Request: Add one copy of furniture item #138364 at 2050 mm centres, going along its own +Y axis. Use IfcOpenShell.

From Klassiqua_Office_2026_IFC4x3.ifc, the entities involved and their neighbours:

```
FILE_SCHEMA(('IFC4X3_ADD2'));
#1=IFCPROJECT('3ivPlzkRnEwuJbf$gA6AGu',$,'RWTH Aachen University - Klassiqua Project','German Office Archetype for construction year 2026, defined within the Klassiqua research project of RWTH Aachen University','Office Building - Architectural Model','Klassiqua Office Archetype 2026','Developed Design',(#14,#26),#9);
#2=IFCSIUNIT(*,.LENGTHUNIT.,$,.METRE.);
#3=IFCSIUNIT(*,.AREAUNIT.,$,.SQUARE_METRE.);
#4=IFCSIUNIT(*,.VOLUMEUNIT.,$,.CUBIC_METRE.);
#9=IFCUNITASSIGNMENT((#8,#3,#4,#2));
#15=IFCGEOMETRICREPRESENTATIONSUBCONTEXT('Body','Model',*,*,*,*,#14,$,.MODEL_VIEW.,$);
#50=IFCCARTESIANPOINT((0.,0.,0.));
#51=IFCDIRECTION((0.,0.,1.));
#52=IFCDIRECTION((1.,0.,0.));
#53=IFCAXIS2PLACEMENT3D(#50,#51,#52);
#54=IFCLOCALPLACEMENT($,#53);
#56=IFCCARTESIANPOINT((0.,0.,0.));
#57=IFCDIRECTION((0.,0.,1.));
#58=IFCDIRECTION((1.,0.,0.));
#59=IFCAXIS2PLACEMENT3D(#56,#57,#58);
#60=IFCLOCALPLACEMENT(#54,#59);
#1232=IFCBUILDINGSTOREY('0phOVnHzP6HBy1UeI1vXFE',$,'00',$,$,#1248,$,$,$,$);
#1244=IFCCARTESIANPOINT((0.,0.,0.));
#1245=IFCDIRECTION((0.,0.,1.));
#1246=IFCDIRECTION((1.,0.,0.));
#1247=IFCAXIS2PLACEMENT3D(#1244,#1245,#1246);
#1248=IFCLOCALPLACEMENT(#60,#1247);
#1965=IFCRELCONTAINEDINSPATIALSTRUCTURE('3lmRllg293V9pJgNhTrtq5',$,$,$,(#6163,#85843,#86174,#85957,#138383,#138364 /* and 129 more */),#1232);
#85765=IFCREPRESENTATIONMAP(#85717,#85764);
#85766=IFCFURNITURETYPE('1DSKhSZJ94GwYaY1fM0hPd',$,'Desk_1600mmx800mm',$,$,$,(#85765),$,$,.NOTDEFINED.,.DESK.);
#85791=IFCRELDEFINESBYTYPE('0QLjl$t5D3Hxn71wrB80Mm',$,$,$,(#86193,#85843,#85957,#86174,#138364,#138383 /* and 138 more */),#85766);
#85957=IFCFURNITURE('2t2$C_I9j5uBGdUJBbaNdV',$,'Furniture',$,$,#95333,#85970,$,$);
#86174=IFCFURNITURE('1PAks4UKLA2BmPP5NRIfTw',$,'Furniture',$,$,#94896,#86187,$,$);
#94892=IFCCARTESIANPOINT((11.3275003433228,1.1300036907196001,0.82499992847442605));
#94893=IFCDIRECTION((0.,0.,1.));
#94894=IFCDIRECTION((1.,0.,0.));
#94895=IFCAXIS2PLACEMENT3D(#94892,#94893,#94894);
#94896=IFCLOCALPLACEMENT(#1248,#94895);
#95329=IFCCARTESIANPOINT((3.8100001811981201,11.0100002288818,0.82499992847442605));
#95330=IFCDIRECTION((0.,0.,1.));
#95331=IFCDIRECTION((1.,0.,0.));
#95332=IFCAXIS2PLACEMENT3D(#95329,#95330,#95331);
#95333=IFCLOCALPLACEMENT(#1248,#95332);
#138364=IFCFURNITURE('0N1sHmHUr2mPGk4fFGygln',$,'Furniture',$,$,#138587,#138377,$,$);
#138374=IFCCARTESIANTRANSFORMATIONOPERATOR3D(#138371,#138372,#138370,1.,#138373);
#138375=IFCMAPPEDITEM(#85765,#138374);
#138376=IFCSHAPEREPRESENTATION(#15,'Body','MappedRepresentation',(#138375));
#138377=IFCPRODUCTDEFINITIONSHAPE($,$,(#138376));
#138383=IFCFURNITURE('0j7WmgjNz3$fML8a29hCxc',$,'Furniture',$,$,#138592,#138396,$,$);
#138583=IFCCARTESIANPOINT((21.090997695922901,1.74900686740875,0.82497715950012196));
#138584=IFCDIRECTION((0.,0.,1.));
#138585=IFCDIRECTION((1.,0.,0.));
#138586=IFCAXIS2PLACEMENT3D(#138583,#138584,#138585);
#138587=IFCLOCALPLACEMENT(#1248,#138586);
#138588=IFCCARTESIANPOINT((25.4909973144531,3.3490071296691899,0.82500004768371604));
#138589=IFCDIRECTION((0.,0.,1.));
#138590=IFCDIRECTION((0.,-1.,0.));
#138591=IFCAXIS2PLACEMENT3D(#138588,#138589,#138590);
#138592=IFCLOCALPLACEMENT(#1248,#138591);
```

```python
import ifcopenshell
import ifcopenshell.api.geometry
import ifcopenshell.api.root
import ifcopenshell.util.element
import ifcopenshell.util.placement
import ifcopenshell.util.unit

model = ifcopenshell.open("Klassiqua_Office_2026_IFC4x3.ifc")
unit_scale = ifcopenshell.util.unit.calculate_unit_scale(model)

source = model.by_guid("0N1sHmHUr2mPGk4fFGygln")
base = ifcopenshell.util.placement.get_local_placement(source.ObjectPlacement)
step = base[:3, 1] * 2.05 / unit_scale

for i in range(1, 2):
    copy = ifcopenshell.api.root.copy_class(model, product=source)
    copy.Representation = ifcopenshell.util.element.copy_deep(
        model, source.Representation, exclude=["IfcGeometricRepresentationContext", "IfcRepresentationMap"]
    )
    matrix = base.copy()
    matrix[:3, 3] += i * step
    print("added at", matrix[:3, 3].round(3) + 0.0)
    ifcopenshell.api.geometry.edit_object_placement(model, product=copy, matrix=matrix, is_si=False)

model.write("Klassiqua_Office_2026_IFC4x3_rev.ifc")
```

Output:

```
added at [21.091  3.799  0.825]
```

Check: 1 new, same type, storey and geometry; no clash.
